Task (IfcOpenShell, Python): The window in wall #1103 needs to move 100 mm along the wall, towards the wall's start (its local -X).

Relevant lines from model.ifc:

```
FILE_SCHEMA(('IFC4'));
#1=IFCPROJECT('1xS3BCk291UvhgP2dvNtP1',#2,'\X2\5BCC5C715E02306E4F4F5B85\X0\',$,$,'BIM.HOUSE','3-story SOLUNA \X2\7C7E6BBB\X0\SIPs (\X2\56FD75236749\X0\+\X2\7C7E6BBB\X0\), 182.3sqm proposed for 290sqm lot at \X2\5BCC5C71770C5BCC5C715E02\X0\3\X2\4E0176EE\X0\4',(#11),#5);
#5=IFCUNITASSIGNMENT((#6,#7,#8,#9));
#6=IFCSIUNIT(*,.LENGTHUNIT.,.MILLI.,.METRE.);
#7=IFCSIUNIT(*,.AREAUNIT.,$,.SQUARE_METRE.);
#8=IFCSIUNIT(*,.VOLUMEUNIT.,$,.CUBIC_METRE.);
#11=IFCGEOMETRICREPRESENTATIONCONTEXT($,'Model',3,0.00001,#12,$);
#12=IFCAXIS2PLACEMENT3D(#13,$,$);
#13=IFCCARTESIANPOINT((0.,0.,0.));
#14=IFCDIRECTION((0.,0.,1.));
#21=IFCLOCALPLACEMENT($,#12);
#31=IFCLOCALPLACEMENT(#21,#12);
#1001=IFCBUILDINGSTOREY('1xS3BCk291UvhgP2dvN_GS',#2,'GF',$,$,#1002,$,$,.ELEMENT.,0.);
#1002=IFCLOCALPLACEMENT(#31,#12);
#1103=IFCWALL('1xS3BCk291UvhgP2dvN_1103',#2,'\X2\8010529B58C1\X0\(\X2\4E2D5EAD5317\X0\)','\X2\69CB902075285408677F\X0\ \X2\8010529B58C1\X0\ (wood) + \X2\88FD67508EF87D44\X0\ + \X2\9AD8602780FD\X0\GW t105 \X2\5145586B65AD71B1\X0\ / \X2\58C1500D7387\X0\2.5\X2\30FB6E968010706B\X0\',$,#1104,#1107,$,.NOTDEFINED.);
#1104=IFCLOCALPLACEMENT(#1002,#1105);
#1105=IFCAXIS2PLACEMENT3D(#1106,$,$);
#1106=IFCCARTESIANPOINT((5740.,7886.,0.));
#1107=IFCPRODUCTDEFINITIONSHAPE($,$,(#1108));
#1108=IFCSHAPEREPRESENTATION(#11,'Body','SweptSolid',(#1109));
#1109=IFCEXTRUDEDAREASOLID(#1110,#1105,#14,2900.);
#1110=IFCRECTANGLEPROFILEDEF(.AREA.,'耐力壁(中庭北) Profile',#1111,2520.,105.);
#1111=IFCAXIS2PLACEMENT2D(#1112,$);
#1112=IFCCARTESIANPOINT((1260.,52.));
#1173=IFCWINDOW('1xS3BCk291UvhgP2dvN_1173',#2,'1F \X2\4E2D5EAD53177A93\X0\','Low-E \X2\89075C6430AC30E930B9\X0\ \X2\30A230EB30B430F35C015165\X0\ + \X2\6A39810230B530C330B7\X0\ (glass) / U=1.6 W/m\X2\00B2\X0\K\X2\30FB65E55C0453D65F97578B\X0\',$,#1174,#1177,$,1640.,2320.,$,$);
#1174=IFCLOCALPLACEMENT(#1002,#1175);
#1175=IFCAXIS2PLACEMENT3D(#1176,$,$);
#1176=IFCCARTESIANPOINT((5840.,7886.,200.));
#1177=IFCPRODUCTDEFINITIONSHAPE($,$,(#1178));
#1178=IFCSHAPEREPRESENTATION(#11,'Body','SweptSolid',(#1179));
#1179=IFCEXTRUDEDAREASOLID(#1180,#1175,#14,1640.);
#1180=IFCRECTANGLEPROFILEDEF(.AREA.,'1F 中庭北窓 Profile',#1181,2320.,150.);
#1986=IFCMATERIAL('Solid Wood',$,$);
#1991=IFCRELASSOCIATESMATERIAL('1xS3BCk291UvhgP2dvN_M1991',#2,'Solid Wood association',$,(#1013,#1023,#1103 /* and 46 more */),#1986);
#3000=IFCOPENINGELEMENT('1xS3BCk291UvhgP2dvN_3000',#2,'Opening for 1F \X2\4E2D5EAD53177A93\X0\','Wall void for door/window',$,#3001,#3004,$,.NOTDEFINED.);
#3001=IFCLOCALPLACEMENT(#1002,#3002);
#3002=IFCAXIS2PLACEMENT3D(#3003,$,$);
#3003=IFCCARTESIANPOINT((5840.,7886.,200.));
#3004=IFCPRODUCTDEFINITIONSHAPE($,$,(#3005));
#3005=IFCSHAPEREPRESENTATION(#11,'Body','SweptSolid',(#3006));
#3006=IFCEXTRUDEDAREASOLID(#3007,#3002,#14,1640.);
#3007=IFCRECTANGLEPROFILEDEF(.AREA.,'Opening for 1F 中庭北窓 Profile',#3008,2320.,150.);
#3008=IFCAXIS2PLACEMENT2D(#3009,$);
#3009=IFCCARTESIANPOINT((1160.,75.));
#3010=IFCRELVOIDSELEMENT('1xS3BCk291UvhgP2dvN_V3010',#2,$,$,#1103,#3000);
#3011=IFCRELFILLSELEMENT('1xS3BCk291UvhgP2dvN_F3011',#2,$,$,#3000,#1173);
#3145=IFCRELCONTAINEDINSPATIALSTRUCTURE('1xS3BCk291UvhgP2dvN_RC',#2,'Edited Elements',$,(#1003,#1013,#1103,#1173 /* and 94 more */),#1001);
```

```python
import ifcopenshell
import ifcopenshell.api.geometry
import ifcopenshell.util.placement

model = ifcopenshell.open("model.ifc")

window = model.by_guid("1xS3BCk291UvhgP2dvN_1173")
opening = window.FillsVoids[0].RelatingOpeningElement
wall = opening.VoidsElements[0].RelatingBuildingElement

wall_matrix = ifcopenshell.util.placement.get_local_placement(wall.ObjectPlacement)
shift = wall_matrix[:3, 0] * -100.0
before = ifcopenshell.util.placement.get_local_placement(window.ObjectPlacement)[:3, 3].copy()

# The window is not placed relative to its opening, so move both.
for product in (opening, window):
    matrix = ifcopenshell.util.placement.get_local_placement(product.ObjectPlacement)
    matrix[:3, 3] += shift
    ifcopenshell.api.geometry.edit_object_placement(model, product=product, matrix=matrix, is_si=False)

after = ifcopenshell.util.placement.get_local_placement(window.ObjectPlacement)[:3, 3]
print("window moved by", (after - before).round(3) + 0.0)

model.write("model_updated.ifc")
```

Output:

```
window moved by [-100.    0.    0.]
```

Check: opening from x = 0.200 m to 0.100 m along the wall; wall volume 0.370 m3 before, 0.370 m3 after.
